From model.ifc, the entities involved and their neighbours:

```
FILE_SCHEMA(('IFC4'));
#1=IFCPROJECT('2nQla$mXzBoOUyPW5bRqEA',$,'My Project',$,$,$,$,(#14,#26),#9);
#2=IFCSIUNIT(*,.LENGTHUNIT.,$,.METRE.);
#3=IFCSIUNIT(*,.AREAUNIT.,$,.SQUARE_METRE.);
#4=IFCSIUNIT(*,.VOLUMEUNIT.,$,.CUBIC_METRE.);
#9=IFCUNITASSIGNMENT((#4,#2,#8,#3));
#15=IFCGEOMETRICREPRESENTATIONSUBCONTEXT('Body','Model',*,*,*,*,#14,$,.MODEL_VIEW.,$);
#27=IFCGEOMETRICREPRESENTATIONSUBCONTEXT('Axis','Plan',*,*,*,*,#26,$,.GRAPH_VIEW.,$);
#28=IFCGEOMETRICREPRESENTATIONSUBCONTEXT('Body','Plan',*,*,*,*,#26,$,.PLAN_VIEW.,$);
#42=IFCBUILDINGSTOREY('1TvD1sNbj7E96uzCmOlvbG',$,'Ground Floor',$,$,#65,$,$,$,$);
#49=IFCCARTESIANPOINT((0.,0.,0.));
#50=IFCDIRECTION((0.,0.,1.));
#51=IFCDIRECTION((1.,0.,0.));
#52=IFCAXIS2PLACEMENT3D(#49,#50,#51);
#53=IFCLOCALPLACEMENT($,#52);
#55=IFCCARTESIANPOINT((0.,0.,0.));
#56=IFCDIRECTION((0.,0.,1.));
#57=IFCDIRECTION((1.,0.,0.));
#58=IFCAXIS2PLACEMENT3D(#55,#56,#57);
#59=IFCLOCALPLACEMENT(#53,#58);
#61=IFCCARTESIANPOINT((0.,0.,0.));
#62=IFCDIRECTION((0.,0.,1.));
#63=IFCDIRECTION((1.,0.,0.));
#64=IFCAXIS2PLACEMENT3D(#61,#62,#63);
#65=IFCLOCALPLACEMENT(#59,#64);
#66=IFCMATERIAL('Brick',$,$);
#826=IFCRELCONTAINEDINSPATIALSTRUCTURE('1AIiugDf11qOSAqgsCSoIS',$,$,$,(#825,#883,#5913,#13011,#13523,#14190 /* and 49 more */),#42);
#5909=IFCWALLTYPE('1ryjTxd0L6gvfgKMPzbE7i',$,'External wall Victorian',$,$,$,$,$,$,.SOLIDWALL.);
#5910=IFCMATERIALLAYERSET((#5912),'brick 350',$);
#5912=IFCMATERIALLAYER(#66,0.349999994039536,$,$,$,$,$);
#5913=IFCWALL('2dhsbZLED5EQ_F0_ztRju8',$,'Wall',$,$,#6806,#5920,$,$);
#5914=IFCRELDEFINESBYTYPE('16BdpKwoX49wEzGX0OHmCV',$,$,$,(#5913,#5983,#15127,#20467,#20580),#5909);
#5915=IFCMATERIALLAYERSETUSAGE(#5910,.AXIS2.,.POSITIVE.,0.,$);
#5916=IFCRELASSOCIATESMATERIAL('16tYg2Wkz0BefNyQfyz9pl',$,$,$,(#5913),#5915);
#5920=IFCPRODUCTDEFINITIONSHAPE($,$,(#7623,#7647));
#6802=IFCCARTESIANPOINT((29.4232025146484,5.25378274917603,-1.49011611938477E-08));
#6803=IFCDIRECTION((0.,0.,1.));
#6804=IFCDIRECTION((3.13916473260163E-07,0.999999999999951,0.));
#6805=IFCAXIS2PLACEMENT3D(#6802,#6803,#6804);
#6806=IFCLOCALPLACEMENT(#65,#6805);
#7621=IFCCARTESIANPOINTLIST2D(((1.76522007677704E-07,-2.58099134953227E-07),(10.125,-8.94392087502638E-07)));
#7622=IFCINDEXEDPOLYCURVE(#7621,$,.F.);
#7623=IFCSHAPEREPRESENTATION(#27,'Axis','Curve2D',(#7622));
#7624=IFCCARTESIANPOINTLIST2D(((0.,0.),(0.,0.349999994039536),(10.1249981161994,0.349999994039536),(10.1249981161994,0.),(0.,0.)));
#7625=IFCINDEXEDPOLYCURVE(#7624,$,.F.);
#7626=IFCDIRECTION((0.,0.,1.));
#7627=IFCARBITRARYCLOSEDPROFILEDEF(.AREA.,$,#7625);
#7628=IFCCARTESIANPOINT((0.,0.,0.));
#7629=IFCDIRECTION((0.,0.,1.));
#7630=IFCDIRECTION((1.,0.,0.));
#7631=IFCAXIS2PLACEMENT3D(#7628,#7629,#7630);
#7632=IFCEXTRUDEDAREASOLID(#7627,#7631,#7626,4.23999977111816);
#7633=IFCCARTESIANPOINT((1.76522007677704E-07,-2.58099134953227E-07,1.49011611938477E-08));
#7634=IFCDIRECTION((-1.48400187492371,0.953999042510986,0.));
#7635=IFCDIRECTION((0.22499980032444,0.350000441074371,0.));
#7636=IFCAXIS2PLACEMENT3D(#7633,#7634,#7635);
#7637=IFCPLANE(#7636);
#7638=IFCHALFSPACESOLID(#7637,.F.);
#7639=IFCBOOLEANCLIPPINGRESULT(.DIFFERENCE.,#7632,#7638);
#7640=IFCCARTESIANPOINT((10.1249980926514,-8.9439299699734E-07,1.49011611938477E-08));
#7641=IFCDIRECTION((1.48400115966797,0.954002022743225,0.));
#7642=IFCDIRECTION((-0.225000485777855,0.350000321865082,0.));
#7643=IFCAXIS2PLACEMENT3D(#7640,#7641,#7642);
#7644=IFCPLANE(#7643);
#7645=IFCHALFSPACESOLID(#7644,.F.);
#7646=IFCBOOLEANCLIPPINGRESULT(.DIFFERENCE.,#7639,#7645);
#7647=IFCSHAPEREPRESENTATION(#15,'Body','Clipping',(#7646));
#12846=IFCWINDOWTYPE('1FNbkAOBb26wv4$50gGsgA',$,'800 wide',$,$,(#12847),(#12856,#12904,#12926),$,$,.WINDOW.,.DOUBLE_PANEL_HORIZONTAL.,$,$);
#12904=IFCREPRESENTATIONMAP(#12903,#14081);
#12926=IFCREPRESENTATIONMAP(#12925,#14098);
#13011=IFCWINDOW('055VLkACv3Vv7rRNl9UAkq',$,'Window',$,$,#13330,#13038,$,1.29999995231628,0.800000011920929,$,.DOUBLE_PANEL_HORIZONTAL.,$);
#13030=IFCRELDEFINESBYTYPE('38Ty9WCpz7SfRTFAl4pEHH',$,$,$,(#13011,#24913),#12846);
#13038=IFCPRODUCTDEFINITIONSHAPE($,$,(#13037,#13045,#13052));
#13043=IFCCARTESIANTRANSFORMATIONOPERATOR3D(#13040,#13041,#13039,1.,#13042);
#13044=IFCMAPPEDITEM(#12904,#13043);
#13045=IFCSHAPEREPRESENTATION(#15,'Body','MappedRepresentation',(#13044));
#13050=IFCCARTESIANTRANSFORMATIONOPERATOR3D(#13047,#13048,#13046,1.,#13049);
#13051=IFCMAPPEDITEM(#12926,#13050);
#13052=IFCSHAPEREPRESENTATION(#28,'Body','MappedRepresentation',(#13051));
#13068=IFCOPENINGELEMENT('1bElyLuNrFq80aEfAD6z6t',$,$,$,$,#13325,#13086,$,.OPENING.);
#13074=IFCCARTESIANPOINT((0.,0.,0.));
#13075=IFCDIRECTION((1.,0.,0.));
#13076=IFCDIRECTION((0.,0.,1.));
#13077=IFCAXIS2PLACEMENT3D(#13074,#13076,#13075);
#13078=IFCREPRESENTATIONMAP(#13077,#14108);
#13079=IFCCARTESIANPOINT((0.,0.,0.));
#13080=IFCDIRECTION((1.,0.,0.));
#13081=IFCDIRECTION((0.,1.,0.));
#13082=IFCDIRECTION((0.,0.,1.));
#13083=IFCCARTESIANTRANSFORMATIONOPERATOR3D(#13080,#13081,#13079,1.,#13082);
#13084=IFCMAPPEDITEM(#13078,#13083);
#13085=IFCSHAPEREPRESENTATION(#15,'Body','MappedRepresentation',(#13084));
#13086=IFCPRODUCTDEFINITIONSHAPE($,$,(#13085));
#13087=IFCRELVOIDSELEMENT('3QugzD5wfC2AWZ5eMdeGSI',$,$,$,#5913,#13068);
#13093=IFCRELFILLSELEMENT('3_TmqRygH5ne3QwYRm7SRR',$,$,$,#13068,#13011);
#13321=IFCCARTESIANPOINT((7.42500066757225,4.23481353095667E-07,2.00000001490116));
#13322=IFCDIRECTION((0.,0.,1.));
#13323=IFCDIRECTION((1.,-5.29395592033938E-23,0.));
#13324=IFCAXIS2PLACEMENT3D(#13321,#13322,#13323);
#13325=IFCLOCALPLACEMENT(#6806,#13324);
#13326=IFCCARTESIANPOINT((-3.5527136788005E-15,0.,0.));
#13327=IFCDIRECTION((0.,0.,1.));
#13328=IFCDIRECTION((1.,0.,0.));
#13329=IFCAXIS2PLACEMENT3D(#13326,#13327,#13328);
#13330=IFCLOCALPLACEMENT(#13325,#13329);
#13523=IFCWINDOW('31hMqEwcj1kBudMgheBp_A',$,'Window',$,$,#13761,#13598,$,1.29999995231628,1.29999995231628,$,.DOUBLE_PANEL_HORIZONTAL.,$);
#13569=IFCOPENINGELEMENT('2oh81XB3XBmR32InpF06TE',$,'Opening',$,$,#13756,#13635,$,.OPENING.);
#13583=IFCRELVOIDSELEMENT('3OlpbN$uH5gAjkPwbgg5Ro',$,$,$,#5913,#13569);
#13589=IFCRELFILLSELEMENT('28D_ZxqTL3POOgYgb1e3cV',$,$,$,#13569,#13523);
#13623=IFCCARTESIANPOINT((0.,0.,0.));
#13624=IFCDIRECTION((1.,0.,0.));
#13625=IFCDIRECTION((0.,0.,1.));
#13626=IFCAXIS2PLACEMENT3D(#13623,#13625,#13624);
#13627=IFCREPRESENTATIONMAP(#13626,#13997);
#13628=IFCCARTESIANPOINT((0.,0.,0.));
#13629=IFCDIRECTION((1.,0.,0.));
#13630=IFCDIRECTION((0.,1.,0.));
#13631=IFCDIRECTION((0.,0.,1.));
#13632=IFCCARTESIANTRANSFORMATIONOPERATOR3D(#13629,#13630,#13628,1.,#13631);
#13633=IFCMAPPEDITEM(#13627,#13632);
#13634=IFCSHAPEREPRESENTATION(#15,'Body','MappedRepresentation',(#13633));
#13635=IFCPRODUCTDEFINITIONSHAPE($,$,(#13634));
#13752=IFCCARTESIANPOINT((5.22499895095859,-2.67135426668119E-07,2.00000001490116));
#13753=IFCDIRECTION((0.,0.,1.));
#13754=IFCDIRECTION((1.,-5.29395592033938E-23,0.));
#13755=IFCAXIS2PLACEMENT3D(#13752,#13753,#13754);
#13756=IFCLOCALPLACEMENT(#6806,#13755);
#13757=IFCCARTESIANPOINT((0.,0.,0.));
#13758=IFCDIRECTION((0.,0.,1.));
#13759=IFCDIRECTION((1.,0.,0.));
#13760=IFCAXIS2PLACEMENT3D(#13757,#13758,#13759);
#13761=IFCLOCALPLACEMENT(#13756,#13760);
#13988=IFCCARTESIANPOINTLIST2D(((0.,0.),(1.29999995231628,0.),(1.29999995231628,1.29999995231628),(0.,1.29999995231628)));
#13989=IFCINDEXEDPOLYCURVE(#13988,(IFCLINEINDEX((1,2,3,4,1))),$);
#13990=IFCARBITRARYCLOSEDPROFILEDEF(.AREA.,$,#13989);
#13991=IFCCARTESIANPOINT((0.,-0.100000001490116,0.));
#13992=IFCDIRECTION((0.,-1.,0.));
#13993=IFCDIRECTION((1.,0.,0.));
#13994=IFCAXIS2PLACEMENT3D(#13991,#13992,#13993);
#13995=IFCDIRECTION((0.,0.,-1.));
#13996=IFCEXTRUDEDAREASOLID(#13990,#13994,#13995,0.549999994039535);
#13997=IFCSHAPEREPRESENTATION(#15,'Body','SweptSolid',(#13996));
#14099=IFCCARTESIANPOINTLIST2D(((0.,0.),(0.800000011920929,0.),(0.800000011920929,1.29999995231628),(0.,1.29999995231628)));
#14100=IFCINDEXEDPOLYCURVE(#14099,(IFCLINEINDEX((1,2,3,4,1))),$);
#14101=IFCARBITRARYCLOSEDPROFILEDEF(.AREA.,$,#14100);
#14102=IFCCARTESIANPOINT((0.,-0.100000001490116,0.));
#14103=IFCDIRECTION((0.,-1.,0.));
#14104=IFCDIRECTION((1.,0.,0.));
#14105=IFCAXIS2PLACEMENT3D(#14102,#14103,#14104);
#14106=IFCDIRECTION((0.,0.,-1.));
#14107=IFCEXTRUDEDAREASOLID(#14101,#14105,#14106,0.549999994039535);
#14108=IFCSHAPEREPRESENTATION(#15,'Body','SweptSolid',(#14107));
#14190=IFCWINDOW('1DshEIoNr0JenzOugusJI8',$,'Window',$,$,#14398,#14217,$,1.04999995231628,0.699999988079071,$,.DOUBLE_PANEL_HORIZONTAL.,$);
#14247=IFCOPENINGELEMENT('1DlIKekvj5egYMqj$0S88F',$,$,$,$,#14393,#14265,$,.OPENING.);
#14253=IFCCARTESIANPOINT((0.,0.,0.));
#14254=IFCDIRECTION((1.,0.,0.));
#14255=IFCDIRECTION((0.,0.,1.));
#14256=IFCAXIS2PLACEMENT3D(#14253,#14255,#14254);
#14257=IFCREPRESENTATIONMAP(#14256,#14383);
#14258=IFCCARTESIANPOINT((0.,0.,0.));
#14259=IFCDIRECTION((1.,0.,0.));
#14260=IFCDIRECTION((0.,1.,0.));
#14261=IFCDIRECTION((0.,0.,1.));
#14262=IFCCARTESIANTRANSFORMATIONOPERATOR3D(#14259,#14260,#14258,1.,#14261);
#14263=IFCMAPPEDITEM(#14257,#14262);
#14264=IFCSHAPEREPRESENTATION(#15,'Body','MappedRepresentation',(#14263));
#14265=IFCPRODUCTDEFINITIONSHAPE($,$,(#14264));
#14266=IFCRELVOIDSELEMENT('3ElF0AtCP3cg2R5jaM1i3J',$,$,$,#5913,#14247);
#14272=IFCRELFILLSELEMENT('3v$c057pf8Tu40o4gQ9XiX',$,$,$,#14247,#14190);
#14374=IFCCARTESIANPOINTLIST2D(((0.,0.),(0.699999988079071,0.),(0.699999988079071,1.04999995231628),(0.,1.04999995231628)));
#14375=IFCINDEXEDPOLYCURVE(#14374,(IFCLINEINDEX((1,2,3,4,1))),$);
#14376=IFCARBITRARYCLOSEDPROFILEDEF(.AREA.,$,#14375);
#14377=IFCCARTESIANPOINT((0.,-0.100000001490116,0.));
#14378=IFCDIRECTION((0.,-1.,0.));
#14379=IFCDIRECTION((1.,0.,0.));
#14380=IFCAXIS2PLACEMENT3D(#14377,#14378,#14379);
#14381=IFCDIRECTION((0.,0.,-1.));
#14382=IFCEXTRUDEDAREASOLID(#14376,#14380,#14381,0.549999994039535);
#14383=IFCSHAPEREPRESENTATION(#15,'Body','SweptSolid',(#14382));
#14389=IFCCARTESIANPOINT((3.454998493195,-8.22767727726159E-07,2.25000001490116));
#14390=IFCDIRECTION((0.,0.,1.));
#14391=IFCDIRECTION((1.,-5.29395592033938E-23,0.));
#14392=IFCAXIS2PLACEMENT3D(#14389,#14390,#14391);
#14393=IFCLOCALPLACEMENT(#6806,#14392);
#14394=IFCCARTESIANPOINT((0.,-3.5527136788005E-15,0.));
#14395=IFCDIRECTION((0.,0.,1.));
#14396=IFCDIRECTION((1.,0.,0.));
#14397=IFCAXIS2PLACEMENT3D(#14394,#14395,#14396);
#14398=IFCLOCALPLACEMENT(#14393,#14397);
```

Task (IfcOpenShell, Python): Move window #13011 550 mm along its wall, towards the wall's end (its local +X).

```python
import ifcopenshell
import ifcopenshell.api.geometry
import ifcopenshell.util.placement
import ifcopenshell.util.unit

model = ifcopenshell.open("model.ifc")
unit_scale = ifcopenshell.util.unit.calculate_unit_scale(model)

window = model.by_id(13011)
opening = window.FillsVoids[0].RelatingOpeningElement
wall = opening.VoidsElements[0].RelatingBuildingElement

wall_matrix = ifcopenshell.util.placement.get_local_placement(wall.ObjectPlacement)
shift = wall_matrix[:3, 0] * 0.55 / unit_scale
before = ifcopenshell.util.placement.get_local_placement(window.ObjectPlacement)[:3, 3].copy()

# The window is placed relative to its opening, so it follows when the opening moves.
matrix = ifcopenshell.util.placement.get_local_placement(opening.ObjectPlacement)
matrix[:3, 3] += shift
ifcopenshell.api.geometry.edit_object_placement(
    model, product=opening, matrix=matrix, is_si=False, should_transform_children=True
)

after = ifcopenshell.util.placement.get_local_placement(window.ObjectPlacement)[:3, 3]
print("window moved by", (after - before).round(3) + 0.0)

model.write("model_updated.ifc")
```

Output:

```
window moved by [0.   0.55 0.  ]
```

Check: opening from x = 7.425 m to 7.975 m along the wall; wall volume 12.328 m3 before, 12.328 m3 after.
